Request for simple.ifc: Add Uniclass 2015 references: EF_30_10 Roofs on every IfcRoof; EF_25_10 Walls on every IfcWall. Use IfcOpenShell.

First a look at what the model holds.

```python
import ifcopenshell

model = ifcopenshell.open("simple.ifc")
print(model.schema)
print("classifications:", [c.Name for c in model.by_type("IfcClassification")])
for ifc_class in ("IfcDoor", "IfcRoof", "IfcStair", "IfcWall", "IfcWindow"):
    print(ifc_class, len(model.by_type(ifc_class)))
```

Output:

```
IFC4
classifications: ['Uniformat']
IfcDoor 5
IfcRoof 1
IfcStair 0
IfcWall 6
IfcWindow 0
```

```python
import ifcopenshell
import ifcopenshell.api.classification

model = ifcopenshell.open("simple.ifc")

system = ifcopenshell.api.classification.add_classification(model, classification="Uniclass 2015")

codes = {
    "IfcRoof": ("EF_30_10", "Roofs"),
    "IfcWall": ("EF_25_10", "Walls"),
}
for ifc_class, (code, name) in codes.items():
    products = model.by_type(ifc_class)
    ifcopenshell.api.classification.add_reference(
        model, products=products, classification=system, identification=code, name=name
    )
    print(code, len(products))

model.write("simple_edited.ifc")
```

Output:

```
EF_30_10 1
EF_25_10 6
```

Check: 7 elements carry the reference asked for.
